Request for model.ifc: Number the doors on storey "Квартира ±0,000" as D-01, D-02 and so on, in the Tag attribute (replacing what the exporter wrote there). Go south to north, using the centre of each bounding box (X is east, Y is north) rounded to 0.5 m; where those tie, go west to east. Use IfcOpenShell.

First a look at what the model holds.

```python
import ifcopenshell
import ifcopenshell.util.element
import ifcopenshell.util.placement

model = ifcopenshell.open("model.ifc")
print(model.schema)
storey = next(s for s in model.by_type("IfcBuildingStorey") if s.Name == "Квартира ±0,000")
doors = [e for e in ifcopenshell.util.element.get_decomposition(storey) if e.is_a("IfcDoor")]
for e in sorted(doors, key=lambda e: e.id()):
    origin = ifcopenshell.util.placement.get_local_placement(e.ObjectPlacement)[:3, 3]
    print(e.id(), e.Tag, e.Name, origin.round(2) + 0.0, sep=" | ")
```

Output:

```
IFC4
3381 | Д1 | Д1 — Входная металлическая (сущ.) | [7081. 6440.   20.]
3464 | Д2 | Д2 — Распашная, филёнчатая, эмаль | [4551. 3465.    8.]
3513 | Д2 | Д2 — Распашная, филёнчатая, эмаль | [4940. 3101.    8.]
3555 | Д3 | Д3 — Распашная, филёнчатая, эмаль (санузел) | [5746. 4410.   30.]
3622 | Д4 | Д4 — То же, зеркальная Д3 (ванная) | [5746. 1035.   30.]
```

```python
import ifcopenshell
import ifcopenshell.geom
import ifcopenshell.util.element
import ifcopenshell.util.shape

model = ifcopenshell.open("model.ifc")
settings = ifcopenshell.geom.settings()
settings.set("use-world-coords", True)


def centre(element):
    shape = ifcopenshell.geom.create_shape(settings, element)
    return ifcopenshell.util.shape.get_bbox_centroid(shape.geometry)


storey = next(s for s in model.by_type("IfcBuildingStorey") if s.Name == "Квартира ±0,000")
doors = [e for e in ifcopenshell.util.element.get_decomposition(storey) if e.is_a("IfcDoor")]

# Insertion points can sit at a corner or the storey origin, so sort by the geometry (in metres).
centres = {e: centre(e) for e in doors}
doors.sort(key=lambda e: (round(centres[e][1] / 0.5), centres[e][0]))

for i, e in enumerate(doors, start=1):
    number = f"D-{i:02d}"
    e.Tag = number
    print(e.id(), number)

model.write("model_v2.ifc")
```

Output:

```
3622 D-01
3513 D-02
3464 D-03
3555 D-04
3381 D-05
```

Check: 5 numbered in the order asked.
